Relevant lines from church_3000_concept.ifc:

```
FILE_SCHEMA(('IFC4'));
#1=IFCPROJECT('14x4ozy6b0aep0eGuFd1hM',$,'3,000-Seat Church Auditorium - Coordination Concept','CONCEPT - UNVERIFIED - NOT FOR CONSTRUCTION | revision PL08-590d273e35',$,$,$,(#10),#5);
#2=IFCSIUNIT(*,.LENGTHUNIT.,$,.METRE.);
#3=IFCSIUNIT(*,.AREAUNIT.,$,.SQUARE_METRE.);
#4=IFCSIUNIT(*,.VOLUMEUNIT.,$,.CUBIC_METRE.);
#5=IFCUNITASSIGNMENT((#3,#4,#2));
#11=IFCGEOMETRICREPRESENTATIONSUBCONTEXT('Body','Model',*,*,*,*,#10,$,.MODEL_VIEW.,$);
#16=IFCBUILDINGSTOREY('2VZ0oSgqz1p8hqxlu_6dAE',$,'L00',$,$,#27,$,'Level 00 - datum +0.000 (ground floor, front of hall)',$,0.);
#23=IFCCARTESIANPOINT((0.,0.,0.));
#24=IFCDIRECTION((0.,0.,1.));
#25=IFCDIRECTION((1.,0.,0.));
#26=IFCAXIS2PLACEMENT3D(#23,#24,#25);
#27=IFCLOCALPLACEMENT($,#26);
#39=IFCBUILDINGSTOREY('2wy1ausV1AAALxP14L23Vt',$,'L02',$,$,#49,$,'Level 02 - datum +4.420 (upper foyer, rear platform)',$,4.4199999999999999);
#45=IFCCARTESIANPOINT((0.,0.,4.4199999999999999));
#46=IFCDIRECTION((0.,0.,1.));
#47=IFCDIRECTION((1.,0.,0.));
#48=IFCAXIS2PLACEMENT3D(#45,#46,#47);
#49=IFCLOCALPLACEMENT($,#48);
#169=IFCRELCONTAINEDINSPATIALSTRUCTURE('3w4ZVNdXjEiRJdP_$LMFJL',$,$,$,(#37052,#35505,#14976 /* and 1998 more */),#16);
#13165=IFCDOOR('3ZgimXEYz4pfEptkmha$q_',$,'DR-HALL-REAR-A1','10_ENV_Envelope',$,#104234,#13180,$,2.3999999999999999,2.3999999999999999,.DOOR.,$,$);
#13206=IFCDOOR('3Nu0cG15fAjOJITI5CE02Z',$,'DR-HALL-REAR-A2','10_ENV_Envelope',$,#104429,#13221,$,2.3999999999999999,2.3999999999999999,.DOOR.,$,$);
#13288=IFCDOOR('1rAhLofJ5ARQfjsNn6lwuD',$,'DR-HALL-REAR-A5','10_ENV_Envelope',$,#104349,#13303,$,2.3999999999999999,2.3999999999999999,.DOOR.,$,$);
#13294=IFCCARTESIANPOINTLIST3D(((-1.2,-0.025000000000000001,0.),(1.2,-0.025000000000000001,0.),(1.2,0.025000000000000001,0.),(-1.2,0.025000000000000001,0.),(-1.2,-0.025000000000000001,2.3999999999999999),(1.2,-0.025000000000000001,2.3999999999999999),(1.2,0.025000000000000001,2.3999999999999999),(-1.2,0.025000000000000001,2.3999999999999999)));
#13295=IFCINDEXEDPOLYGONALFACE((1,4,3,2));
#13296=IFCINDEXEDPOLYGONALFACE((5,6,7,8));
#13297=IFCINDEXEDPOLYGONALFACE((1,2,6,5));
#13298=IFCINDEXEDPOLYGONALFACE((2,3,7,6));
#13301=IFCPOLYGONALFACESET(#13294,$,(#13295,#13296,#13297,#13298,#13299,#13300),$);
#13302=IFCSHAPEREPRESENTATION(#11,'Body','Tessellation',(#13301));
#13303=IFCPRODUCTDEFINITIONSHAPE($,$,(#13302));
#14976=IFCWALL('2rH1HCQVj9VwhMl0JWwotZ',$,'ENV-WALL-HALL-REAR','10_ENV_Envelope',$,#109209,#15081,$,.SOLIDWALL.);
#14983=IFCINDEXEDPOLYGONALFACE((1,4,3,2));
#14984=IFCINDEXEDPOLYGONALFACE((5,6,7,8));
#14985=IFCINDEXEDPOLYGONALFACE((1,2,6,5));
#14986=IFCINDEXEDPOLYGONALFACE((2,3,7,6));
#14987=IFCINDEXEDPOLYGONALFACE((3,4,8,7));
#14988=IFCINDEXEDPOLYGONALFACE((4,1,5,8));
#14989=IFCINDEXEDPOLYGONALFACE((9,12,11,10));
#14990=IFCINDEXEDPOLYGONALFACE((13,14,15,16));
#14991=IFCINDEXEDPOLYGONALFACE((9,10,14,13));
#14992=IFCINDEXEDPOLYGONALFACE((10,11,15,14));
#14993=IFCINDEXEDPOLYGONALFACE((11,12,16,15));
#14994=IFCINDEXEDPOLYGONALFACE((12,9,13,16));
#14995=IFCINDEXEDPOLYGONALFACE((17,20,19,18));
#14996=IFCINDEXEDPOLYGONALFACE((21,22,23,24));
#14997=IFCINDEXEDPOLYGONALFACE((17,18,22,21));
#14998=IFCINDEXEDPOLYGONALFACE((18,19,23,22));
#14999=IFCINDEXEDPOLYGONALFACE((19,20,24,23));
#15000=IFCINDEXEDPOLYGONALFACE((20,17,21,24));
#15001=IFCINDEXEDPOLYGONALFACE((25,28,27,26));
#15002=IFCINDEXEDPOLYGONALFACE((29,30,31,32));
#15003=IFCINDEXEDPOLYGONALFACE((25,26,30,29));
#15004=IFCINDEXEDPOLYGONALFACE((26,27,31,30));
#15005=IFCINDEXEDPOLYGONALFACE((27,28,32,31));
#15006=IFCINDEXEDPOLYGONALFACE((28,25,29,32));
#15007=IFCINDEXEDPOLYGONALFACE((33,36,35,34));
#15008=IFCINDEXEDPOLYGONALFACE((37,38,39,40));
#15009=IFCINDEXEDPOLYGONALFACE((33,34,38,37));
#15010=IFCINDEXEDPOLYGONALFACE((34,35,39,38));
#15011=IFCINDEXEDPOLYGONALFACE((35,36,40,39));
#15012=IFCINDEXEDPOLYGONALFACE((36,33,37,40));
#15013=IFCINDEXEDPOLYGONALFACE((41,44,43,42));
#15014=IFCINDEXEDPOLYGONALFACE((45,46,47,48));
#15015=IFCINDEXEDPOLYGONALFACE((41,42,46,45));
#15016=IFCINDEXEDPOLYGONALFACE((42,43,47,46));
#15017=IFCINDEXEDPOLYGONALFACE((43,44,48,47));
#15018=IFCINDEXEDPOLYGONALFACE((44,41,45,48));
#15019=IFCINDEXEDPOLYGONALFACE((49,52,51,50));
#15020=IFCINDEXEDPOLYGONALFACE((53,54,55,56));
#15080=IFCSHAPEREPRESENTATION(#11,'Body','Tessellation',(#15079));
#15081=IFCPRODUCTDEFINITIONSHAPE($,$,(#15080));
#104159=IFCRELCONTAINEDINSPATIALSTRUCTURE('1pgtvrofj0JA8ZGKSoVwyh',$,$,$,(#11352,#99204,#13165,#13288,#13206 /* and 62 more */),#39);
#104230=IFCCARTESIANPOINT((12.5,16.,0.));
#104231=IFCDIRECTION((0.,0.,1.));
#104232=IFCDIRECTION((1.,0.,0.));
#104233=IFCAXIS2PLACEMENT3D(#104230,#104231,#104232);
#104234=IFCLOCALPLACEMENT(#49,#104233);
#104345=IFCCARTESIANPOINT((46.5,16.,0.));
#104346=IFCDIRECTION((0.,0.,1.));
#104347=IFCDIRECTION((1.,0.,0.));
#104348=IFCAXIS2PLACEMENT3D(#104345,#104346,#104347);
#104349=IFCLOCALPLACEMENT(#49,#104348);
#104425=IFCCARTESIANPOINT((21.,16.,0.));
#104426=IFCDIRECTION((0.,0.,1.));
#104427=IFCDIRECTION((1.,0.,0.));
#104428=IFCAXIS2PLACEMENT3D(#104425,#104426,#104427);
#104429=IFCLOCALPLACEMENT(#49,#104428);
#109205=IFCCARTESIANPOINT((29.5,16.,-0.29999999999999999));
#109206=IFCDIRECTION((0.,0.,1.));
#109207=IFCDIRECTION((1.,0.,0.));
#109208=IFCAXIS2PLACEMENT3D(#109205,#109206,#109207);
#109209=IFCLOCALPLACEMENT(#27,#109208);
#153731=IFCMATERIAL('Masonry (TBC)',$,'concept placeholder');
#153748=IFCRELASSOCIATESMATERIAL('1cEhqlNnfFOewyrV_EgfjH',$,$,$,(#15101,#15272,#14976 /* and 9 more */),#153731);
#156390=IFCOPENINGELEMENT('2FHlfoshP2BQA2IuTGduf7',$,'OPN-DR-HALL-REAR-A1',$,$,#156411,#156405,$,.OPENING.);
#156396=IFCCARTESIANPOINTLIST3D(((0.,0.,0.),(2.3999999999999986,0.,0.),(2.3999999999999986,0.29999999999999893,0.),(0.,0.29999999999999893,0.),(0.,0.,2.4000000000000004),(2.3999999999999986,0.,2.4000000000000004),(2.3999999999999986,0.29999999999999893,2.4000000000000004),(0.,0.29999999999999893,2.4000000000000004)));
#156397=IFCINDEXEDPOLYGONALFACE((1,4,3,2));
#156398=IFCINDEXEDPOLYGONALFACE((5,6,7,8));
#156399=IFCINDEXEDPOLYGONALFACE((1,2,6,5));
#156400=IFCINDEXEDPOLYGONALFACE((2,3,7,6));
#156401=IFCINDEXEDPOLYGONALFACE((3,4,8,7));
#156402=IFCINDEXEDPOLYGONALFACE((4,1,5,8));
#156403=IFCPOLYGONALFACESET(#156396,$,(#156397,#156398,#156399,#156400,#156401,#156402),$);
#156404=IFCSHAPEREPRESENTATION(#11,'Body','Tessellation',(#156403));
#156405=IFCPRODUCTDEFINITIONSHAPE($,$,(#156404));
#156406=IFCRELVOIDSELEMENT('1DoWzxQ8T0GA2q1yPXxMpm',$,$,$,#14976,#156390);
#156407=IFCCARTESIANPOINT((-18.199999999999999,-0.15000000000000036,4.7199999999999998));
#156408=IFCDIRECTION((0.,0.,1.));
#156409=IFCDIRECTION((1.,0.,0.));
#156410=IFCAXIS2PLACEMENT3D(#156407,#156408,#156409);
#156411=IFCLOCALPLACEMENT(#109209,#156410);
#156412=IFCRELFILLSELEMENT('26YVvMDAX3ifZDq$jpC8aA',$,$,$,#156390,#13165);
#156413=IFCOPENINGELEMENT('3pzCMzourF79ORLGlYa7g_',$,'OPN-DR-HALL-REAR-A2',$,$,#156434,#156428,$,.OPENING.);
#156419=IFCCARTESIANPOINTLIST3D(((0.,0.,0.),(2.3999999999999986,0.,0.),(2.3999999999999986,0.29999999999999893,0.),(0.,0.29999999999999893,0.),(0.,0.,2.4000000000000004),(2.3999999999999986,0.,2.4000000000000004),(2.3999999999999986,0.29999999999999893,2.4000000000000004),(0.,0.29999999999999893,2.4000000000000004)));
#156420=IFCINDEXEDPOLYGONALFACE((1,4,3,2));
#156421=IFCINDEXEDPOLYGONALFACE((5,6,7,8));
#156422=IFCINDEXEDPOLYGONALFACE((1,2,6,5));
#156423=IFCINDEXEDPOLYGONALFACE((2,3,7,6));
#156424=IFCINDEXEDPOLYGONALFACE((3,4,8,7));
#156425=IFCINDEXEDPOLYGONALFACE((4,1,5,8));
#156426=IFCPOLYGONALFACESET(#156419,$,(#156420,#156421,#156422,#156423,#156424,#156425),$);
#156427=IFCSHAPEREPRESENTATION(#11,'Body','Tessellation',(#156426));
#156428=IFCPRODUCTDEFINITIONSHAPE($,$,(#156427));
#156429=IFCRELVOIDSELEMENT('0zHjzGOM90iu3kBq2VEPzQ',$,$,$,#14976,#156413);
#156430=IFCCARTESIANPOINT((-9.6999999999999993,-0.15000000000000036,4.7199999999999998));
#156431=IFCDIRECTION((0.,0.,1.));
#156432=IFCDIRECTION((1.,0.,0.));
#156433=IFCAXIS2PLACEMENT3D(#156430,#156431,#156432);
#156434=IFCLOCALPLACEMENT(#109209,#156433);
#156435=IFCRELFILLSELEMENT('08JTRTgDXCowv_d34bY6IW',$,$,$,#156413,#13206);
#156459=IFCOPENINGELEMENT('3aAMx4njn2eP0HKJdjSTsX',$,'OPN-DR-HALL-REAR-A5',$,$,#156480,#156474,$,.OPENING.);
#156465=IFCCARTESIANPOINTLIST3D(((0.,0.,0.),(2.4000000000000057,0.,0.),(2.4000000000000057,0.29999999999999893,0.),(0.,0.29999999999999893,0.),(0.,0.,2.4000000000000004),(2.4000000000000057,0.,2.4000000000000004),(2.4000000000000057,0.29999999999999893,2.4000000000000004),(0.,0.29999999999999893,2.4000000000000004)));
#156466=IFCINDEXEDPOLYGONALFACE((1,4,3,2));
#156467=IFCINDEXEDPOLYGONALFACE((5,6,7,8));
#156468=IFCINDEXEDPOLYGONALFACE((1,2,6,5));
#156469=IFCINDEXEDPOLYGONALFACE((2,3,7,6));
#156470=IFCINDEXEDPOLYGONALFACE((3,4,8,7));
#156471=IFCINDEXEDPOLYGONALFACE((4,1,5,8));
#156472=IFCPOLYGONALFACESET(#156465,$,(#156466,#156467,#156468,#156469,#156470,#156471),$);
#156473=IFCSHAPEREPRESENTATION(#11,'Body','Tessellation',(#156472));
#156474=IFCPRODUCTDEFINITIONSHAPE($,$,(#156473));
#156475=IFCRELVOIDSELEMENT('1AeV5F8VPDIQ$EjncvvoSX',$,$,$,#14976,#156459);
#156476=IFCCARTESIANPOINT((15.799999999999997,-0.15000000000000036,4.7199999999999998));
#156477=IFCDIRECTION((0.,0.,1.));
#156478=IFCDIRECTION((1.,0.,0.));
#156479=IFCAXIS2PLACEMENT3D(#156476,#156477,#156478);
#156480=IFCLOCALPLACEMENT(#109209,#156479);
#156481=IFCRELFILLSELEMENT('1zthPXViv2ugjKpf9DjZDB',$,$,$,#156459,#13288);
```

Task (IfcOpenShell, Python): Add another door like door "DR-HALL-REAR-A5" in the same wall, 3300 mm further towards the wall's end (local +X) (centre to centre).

```python
import ifcopenshell
import ifcopenshell.api.feature
import ifcopenshell.api.geometry
import ifcopenshell.api.root
import ifcopenshell.geom
import ifcopenshell.util.element
import ifcopenshell.util.placement
import ifcopenshell.util.shape
import ifcopenshell.util.unit

model = ifcopenshell.open("church_3000_concept.ifc")
unit_scale = ifcopenshell.util.unit.calculate_unit_scale(model)
settings = ifcopenshell.geom.settings()


def volume(element):
    """Net volume in cubic metres, openings subtracted."""
    shape = ifcopenshell.geom.create_shape(settings, element)
    return ifcopenshell.util.shape.get_volume(shape.geometry)


door = model.by_id(13288)
opening = door.FillsVoids[0].RelatingOpeningElement
wall = opening.VoidsElements[0].RelatingBuildingElement
before = volume(wall)
shift = ifcopenshell.util.placement.get_local_placement(wall.ObjectPlacement)[:3, 0] * 3.3 / unit_scale

# copy_class copies the void relationship, type, container and properties, but no geometry.
new_opening = ifcopenshell.api.root.copy_class(model, product=opening)
new_opening.Representation = ifcopenshell.util.element.copy_deep(
    model, opening.Representation, exclude=["IfcGeometricRepresentationContext", "IfcRepresentationMap"]
)
new_door = ifcopenshell.api.root.copy_class(model, product=door)
new_door.Representation = ifcopenshell.util.element.copy_deep(
    model, door.Representation, exclude=["IfcGeometricRepresentationContext", "IfcRepresentationMap"]
)
ifcopenshell.api.feature.add_filling(model, opening=new_opening, element=new_door)

for old, new in ((opening, new_opening), (door, new_door)):
    matrix = ifcopenshell.util.placement.get_local_placement(old.ObjectPlacement)
    matrix[:3, 3] += shift
    ifcopenshell.api.geometry.edit_object_placement(model, product=new, matrix=matrix, is_si=False)

after = volume(wall)

print(f"wall volume {before:.3f} -> {after:.3f} m3")

model.write("church_3000_concept-out.ifc")
```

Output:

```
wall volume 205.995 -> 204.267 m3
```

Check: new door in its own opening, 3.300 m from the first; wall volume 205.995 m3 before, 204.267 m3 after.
